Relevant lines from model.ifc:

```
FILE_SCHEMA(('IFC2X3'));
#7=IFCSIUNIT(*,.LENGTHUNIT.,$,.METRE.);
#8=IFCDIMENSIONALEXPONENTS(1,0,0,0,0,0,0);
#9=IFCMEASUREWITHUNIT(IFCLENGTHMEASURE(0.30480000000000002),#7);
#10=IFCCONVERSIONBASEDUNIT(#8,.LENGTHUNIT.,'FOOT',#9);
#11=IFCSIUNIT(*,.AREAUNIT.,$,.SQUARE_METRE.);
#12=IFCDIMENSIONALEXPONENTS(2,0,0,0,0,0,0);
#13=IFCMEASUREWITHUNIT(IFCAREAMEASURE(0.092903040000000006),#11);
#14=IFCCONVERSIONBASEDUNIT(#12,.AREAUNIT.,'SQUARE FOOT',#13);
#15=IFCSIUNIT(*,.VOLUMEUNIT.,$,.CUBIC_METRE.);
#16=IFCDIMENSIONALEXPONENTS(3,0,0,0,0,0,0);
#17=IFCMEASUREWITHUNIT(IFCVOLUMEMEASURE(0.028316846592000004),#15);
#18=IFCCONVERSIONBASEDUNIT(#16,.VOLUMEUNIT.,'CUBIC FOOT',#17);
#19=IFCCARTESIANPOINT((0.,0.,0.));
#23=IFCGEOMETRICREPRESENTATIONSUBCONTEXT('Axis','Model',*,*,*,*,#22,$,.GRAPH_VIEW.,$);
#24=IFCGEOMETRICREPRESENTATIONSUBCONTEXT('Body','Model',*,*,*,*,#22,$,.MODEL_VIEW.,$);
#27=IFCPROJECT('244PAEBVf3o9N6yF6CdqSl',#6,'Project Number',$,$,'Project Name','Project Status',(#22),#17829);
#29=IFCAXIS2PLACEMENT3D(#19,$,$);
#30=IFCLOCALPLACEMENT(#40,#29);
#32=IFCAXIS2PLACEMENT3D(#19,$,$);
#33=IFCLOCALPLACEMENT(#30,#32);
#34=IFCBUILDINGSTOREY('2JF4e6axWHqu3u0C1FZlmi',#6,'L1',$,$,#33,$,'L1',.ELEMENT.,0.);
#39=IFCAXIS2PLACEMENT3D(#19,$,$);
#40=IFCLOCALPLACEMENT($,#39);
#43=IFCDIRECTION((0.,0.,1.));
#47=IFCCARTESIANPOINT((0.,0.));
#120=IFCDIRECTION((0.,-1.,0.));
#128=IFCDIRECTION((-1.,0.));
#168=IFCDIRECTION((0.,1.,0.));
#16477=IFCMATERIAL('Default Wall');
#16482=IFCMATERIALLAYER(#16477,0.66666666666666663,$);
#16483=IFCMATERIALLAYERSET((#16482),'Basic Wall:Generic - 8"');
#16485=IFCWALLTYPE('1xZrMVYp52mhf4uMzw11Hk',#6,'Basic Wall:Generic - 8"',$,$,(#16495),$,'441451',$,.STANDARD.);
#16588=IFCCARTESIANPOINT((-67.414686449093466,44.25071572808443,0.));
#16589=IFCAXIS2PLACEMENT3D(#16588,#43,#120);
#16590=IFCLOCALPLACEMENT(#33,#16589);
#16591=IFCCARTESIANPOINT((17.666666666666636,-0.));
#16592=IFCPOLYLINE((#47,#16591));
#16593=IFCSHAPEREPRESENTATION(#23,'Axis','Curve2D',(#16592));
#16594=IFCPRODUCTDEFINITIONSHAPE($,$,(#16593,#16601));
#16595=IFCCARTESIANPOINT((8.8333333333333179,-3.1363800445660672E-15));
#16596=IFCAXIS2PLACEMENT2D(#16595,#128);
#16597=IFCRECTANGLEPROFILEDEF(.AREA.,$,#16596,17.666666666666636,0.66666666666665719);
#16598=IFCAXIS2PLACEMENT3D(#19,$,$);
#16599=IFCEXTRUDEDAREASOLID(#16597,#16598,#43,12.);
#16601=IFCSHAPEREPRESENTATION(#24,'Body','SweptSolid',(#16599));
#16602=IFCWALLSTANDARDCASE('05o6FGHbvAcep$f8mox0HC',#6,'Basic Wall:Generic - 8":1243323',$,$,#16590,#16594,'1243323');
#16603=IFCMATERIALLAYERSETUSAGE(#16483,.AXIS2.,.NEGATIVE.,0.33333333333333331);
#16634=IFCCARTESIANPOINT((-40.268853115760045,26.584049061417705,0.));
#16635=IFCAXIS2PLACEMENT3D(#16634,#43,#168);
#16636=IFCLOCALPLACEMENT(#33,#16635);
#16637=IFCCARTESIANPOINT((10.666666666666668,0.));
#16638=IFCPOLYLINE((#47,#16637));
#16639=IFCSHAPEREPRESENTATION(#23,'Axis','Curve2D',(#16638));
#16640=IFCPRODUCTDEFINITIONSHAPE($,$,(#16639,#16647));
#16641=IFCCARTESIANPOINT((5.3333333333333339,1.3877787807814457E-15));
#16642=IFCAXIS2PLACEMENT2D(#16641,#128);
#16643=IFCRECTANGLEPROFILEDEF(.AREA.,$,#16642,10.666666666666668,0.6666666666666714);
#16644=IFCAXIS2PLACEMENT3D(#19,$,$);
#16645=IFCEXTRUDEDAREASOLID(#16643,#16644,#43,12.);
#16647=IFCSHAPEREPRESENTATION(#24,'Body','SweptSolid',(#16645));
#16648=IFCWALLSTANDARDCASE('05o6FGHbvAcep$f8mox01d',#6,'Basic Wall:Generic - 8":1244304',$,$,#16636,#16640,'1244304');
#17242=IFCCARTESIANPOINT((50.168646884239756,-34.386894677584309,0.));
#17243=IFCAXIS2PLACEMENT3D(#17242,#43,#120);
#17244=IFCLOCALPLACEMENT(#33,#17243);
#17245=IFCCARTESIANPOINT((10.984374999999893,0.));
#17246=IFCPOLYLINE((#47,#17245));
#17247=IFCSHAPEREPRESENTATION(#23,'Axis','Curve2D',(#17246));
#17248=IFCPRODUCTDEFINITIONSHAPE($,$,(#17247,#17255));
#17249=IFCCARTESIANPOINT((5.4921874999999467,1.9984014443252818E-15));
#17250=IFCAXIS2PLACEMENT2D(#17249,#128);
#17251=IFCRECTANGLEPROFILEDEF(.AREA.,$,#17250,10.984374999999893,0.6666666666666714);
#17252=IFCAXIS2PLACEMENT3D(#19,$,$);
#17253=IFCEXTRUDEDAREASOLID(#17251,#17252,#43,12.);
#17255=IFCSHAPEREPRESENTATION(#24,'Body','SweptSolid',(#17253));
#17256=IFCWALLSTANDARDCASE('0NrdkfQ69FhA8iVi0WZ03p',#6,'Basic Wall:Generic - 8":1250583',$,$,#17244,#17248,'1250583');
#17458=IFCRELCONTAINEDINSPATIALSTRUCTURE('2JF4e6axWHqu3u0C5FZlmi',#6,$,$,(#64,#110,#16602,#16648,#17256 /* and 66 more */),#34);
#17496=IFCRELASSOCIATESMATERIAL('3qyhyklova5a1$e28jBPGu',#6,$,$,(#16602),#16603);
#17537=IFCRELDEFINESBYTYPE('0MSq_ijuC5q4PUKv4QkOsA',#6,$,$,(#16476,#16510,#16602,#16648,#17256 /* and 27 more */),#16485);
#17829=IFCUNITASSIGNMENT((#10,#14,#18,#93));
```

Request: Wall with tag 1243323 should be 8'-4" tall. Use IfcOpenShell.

```python
import ifcopenshell
import ifcopenshell.geom
import ifcopenshell.util.representation
import ifcopenshell.util.shape
import ifcopenshell.util.unit

model = ifcopenshell.open("model.ifc")
unit_scale = ifcopenshell.util.unit.calculate_unit_scale(model)
settings = ifcopenshell.geom.settings()


def volume(element):
    """Net volume in cubic metres, openings subtracted."""
    shape = ifcopenshell.geom.create_shape(settings, element)
    return ifcopenshell.util.shape.get_volume(shape.geometry)


wall = model.by_id(16602)
before = volume(wall)

body = ifcopenshell.util.representation.get_representation(wall, "Model", "Body")
solid = body.Items[0]
old_height = solid.Depth
solid.Depth = 100 * 0.0254 / unit_scale
after = volume(wall)

print(f"height {old_height:g} -> {solid.Depth:g}, volume {before:.3f} -> {after:.3f} m3")

model.write("model_v2.ifc")
```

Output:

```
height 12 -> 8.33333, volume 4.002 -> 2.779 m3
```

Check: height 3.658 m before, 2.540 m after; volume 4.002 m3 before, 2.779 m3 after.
